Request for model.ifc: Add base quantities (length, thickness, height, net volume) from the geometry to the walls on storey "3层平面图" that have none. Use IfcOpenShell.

First a look at what the model holds.

```python
import ifcopenshell
import ifcopenshell.util.element
import ifcopenshell.util.unit

model = ifcopenshell.open("model.ifc")
print(model.schema)
for unit_type in ("LENGTHUNIT", "AREAUNIT", "VOLUMEUNIT"):
    print(unit_type, ifcopenshell.util.unit.calculate_unit_scale(model, unit_type))
storey = next(s for s in model.by_type("IfcBuildingStorey") if s.Name == "3层平面图")
walls = [e for e in ifcopenshell.util.element.get_decomposition(storey) if e.is_a("IfcWall")]
for e in sorted(walls, key=lambda e: e.id()):
    print(e.id(), e.is_a(), e.Name, list(ifcopenshell.util.element.get_psets(e, qtos_only=True)), sep=" | ")
```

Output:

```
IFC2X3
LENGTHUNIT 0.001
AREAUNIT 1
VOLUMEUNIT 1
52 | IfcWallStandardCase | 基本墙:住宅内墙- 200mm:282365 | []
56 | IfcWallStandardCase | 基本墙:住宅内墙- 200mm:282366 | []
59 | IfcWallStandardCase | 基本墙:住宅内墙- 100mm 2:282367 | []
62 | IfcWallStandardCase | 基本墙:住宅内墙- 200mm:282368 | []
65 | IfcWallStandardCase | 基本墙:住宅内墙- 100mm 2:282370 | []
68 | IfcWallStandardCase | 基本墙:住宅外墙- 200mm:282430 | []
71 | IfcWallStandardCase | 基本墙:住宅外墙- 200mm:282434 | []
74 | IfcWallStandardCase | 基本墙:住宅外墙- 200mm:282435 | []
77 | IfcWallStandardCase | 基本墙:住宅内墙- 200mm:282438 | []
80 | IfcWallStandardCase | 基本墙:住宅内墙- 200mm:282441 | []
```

```python
import ifcopenshell
import ifcopenshell.api.pset
import ifcopenshell.geom
import ifcopenshell.util.element
import ifcopenshell.util.shape
import ifcopenshell.util.unit

model = ifcopenshell.open("model.ifc")
unit_scale = ifcopenshell.util.unit.calculate_unit_scale(model)
volume_scale = ifcopenshell.util.unit.calculate_unit_scale(model, "VOLUMEUNIT")
settings = ifcopenshell.geom.settings()

storey = next(s for s in model.by_type("IfcBuildingStorey") if s.Name == "3层平面图")
walls = [e for e in ifcopenshell.util.element.get_decomposition(storey) if e.is_a("IfcWall")]

for e in sorted(walls, key=lambda e: e.id()):
    if ifcopenshell.util.element.get_psets(e, qtos_only=True, should_inherit=False):
        continue
    # Geometry comes back in metres, in the element's own axes.
    shape = ifcopenshell.geom.create_shape(settings, e)
    values = {
        "Length": ifcopenshell.util.shape.get_x(shape.geometry) / unit_scale,
        "Width": ifcopenshell.util.shape.get_y(shape.geometry) / unit_scale,
        "Height": ifcopenshell.util.shape.get_z(shape.geometry) / unit_scale,
        "NetVolume": ifcopenshell.util.shape.get_volume(shape.geometry) / volume_scale,
    }
    qto = ifcopenshell.api.pset.add_qto(model, product=e, name="BaseQuantities")
    ifcopenshell.api.pset.edit_qto(model, qto=qto, properties=values)
    print(e.id(), {k: round(v, 3) for k, v in values.items()})

model.write("model_v2.ifc")
```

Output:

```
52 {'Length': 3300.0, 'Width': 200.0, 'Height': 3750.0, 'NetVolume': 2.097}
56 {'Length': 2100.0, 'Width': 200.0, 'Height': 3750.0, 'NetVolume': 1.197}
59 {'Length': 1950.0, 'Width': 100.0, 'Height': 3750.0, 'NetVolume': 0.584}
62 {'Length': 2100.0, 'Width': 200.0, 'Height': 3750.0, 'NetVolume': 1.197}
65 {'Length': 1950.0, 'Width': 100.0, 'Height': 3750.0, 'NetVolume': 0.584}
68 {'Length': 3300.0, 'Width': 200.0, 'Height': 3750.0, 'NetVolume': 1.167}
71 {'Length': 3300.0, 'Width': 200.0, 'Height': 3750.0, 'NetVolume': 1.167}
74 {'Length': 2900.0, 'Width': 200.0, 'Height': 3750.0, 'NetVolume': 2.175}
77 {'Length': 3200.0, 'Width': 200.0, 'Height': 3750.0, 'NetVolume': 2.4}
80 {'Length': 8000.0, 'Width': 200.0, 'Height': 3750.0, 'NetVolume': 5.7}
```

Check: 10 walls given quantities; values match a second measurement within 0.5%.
